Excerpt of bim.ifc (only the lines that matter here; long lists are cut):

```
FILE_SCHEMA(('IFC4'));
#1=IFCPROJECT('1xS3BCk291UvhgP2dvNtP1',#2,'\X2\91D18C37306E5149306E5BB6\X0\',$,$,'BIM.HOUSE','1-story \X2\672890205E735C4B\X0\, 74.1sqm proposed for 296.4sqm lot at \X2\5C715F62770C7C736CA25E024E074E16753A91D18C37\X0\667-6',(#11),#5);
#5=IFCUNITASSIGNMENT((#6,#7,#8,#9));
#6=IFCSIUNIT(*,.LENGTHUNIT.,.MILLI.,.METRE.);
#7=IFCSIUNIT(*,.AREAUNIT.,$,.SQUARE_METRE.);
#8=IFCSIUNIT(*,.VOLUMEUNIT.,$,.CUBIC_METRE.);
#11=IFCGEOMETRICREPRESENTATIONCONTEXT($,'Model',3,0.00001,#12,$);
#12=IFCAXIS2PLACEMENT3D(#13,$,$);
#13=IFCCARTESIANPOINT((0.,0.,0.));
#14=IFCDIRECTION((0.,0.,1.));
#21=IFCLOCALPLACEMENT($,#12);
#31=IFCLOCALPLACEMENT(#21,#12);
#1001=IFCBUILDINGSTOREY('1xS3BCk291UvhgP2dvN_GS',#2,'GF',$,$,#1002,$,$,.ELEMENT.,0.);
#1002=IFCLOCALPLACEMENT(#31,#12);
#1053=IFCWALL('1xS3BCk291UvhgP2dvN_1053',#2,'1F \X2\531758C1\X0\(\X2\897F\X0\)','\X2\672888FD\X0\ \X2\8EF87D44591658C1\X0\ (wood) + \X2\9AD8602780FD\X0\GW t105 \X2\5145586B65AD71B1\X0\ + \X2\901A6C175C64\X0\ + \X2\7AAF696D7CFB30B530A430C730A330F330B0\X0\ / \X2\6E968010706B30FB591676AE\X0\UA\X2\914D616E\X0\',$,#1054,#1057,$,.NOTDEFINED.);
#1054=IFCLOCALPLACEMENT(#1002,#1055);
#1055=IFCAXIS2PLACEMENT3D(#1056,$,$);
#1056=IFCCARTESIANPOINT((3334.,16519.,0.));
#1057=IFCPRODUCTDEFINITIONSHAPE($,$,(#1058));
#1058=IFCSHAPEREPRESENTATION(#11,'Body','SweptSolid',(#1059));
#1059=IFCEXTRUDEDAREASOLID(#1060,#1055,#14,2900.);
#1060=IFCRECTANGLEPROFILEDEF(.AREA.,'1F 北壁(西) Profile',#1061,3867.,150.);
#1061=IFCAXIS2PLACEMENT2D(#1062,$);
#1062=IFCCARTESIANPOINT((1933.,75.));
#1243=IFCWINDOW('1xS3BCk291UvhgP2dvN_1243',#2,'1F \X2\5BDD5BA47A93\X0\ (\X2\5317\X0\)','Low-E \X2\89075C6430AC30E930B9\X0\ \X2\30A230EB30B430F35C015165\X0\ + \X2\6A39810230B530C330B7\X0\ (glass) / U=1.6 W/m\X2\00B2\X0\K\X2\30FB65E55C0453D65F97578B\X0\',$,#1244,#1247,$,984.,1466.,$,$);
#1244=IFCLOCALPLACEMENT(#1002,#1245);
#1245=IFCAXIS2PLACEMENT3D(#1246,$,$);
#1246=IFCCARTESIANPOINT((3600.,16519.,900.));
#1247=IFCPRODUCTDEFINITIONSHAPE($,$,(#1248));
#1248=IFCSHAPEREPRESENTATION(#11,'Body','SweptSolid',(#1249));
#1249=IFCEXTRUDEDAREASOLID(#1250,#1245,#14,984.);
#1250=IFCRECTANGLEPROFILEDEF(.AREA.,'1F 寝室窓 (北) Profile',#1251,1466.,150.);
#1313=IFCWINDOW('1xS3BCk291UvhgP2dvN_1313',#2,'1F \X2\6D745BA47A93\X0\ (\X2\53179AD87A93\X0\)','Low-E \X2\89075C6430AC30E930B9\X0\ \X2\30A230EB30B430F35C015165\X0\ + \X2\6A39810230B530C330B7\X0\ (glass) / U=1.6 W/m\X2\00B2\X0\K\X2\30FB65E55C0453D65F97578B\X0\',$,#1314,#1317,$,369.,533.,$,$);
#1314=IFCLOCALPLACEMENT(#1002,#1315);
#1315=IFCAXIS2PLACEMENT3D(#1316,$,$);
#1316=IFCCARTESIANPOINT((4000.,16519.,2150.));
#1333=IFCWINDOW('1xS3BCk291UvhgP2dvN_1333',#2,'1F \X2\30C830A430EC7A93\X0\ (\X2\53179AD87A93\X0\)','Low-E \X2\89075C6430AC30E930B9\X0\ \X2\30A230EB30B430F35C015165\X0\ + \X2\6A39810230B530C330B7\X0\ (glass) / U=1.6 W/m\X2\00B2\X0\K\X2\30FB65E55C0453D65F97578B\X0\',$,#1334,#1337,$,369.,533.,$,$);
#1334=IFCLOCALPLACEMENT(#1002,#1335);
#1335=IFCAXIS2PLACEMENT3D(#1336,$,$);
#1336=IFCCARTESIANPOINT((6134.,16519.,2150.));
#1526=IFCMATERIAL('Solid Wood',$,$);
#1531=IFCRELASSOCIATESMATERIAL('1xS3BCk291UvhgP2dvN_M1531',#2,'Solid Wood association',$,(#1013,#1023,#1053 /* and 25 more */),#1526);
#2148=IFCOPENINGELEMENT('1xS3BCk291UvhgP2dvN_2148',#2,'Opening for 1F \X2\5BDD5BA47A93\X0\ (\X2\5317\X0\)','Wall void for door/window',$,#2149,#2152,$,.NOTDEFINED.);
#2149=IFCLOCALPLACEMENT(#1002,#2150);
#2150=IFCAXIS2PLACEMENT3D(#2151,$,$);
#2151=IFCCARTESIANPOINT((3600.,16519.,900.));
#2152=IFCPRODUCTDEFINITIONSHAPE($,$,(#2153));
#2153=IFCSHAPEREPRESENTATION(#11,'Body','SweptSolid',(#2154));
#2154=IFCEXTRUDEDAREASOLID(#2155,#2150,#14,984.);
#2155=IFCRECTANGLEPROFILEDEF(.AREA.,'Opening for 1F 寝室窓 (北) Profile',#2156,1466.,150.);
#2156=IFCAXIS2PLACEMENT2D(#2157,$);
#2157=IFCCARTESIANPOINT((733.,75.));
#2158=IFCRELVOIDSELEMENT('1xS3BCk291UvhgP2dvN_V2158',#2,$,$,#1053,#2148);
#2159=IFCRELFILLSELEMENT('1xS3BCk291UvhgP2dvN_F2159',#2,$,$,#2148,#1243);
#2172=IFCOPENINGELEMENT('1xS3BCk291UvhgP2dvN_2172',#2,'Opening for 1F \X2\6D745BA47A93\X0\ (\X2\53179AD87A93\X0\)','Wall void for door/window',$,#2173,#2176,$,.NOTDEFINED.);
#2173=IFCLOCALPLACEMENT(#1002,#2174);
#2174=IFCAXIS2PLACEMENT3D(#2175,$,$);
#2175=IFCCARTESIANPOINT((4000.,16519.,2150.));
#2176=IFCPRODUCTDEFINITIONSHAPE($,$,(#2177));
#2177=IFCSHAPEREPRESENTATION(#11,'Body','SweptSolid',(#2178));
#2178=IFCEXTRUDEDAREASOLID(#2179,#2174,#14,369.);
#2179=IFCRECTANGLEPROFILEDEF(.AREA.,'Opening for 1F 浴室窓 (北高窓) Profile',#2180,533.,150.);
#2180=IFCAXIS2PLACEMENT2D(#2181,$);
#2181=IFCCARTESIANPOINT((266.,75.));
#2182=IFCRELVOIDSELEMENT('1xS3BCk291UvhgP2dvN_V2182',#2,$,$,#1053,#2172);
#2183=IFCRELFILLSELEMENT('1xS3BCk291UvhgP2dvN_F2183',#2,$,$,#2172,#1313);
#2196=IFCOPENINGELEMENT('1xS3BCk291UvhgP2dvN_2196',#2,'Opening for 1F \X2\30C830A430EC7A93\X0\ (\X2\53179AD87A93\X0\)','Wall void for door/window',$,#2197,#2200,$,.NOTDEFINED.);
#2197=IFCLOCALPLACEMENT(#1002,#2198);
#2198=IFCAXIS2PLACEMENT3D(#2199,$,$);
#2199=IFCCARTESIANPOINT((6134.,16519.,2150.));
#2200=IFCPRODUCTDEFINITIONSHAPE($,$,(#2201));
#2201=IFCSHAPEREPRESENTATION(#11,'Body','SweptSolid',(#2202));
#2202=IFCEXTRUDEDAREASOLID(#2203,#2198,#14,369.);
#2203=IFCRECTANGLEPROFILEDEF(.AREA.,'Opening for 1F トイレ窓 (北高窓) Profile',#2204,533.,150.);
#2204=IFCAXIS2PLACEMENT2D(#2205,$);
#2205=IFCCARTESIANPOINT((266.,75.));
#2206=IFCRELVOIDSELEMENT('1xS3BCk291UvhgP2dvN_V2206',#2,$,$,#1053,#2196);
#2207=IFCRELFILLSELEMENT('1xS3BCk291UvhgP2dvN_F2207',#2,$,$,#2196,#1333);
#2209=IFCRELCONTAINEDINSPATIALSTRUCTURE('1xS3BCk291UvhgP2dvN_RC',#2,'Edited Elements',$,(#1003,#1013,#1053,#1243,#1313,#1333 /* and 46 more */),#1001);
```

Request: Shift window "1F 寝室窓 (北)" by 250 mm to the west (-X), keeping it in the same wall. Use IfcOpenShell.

```python
import ifcopenshell
import ifcopenshell.api.geometry
import ifcopenshell.util.placement
import ifcopenshell.util.unit

model = ifcopenshell.open("bim.ifc")
unit_scale = ifcopenshell.util.unit.calculate_unit_scale(model)

window = model.by_guid("1xS3BCk291UvhgP2dvN_1243")
opening = window.FillsVoids[0].RelatingOpeningElement
wall = opening.VoidsElements[0].RelatingBuildingElement

wall_matrix = ifcopenshell.util.placement.get_local_placement(wall.ObjectPlacement)
shift = wall_matrix[:3, 0] * -0.25 / unit_scale
before = ifcopenshell.util.placement.get_local_placement(window.ObjectPlacement)[:3, 3].copy()

# The window is not placed relative to its opening, so move both.
for product in (opening, window):
    matrix = ifcopenshell.util.placement.get_local_placement(product.ObjectPlacement)
    matrix[:3, 3] += shift
    ifcopenshell.api.geometry.edit_object_placement(model, product=product, matrix=matrix, is_si=False)

after = ifcopenshell.util.placement.get_local_placement(window.ObjectPlacement)[:3, 3]
print("window moved by", (after - before).round(3) + 0.0)

model.write("bim-out.ifc")
```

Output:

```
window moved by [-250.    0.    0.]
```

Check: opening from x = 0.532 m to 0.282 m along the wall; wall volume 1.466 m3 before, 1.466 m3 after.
